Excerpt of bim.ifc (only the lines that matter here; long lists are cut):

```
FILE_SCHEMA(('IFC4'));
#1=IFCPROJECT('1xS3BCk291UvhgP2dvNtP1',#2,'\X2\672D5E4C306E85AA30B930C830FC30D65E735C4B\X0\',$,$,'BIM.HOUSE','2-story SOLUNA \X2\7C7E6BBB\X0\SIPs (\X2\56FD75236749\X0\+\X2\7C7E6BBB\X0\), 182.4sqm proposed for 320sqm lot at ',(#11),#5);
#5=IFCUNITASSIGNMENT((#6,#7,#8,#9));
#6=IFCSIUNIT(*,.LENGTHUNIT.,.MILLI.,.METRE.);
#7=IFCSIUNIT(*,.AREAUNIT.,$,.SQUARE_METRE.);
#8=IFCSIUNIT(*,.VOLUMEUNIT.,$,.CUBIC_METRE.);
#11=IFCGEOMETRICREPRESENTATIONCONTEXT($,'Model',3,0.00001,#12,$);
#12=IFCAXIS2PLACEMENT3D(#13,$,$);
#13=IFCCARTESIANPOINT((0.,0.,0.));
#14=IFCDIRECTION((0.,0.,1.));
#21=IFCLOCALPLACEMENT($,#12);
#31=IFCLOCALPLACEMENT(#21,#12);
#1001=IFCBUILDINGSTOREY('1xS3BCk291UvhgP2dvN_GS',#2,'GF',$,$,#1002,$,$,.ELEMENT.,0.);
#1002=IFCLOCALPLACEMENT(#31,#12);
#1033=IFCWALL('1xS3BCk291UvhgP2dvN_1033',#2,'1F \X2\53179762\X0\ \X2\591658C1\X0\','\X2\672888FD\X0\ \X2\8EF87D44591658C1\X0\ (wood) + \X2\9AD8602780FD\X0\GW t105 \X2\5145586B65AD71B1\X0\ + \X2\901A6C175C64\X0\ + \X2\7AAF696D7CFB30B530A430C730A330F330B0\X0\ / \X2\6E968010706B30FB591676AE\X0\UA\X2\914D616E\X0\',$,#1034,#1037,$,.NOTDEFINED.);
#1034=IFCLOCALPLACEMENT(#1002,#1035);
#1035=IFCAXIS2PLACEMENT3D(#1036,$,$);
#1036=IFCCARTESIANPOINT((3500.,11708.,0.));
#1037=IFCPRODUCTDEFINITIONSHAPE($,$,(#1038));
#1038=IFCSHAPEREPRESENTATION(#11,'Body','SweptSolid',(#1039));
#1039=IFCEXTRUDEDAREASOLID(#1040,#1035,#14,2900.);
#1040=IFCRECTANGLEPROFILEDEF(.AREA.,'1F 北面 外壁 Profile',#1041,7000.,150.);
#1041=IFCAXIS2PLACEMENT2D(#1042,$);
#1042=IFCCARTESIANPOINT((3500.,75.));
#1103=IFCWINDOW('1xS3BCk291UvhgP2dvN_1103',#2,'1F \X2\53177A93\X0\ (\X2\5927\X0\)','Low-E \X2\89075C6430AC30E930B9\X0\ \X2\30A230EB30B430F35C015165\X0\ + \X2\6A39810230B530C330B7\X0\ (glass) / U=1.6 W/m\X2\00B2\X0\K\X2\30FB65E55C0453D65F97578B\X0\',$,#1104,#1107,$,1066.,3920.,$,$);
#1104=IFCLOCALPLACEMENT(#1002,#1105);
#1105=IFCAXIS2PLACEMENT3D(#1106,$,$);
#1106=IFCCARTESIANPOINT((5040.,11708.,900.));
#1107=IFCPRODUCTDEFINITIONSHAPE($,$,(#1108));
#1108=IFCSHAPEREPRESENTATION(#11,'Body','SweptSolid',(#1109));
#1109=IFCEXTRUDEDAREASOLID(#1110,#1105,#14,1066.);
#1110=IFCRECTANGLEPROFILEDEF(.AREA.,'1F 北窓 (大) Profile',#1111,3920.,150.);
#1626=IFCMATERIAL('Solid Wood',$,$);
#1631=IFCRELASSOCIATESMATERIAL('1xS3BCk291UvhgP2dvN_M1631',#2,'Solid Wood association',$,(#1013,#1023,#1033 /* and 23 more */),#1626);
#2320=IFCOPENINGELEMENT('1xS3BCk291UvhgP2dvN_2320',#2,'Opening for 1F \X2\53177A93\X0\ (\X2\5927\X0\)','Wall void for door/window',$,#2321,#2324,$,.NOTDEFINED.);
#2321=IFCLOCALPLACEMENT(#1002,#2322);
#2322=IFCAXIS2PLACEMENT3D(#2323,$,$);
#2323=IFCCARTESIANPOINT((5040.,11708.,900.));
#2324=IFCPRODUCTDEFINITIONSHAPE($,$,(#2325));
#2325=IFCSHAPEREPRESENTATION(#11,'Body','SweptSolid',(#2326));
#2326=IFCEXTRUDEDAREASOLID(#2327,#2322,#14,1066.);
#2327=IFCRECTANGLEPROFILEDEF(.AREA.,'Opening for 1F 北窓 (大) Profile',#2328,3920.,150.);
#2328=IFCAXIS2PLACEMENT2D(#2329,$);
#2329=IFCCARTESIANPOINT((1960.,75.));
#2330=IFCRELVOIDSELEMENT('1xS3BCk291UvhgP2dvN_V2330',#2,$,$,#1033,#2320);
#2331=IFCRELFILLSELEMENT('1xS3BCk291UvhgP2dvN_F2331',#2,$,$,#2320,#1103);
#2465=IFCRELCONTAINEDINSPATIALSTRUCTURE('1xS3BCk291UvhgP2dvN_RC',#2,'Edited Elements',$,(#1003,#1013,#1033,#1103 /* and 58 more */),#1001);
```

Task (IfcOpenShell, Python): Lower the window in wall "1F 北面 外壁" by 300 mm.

```python
import numpy as np
import ifcopenshell
import ifcopenshell.api.geometry
import ifcopenshell.util.placement
import ifcopenshell.util.unit

model = ifcopenshell.open("bim.ifc")
unit_scale = ifcopenshell.util.unit.calculate_unit_scale(model)

window = model.by_guid("1xS3BCk291UvhgP2dvN_1103")
opening = window.FillsVoids[0].RelatingOpeningElement
dz = -300.0

shift = np.array([0.0, 0.0, dz])
# The window is not placed relative to its opening, so move both.
for product in (opening, window):
    matrix = ifcopenshell.util.placement.get_local_placement(product.ObjectPlacement)
    matrix[:3, 3] += shift
    ifcopenshell.api.geometry.edit_object_placement(model, product=product, matrix=matrix, is_si=False)

print(f"moved by {dz * unit_scale:+.3f} m")

model.write("bim_updated.ifc")
```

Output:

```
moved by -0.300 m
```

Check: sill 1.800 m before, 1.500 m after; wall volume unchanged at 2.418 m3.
